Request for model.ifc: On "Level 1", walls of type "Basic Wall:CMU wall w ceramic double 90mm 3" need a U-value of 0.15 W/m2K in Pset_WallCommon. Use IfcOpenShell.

First a look at what the model holds.

```python
import ifcopenshell
import ifcopenshell.util.element

model = ifcopenshell.open("model.ifc")
print(model.schema)
storey = next(s for s in model.by_type("IfcBuildingStorey") if s.Name == "Level 1")
walls = [e for e in ifcopenshell.util.element.get_decomposition(storey) if e.is_a("IfcWall")]
seen = {}
for e in walls:
    element_type = ifcopenshell.util.element.get_type(e)
    key = (element_type.Name if element_type != e and element_type else None, ifcopenshell.util.element.get_pset(e, "Pset_WallCommon", "ThermalTransmittance"))
    seen[key] = seen.get(key, 0) + 1
for (name, value), count in sorted(seen.items(), key=str):
    print(count, "x", name, "|", value)
```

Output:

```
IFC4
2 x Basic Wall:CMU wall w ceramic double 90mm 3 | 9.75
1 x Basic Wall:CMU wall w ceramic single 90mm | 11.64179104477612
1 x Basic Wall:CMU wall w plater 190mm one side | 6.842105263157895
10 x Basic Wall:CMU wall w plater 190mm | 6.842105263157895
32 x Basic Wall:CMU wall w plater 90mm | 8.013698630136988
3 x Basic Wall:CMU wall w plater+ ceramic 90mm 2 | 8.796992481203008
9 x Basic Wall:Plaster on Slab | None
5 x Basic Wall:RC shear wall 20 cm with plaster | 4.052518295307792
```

```python
import ifcopenshell
import ifcopenshell.api.pset
import ifcopenshell.util.element

model = ifcopenshell.open("model.ifc")

storey = next(s for s in model.by_type("IfcBuildingStorey") if s.Name == "Level 1")
walls = [e for e in ifcopenshell.util.element.get_decomposition(storey) if e.is_a("IfcWall")]

count = 0
for e in walls:
    element_type = ifcopenshell.util.element.get_type(e)
    if element_type in (None, e) or element_type.Name != "Basic Wall:CMU wall w ceramic double 90mm 3":
        continue
    # add_pset returns the element's existing set when there is one.
    pset = ifcopenshell.api.pset.add_pset(model, product=e, name="Pset_WallCommon")
    ifcopenshell.api.pset.edit_pset(model, pset=pset, properties={"ThermalTransmittance": 0.15})
    count += 1

print(count, "walls updated")

model.write("model_edited.ifc")
```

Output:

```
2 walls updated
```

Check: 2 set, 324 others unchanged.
